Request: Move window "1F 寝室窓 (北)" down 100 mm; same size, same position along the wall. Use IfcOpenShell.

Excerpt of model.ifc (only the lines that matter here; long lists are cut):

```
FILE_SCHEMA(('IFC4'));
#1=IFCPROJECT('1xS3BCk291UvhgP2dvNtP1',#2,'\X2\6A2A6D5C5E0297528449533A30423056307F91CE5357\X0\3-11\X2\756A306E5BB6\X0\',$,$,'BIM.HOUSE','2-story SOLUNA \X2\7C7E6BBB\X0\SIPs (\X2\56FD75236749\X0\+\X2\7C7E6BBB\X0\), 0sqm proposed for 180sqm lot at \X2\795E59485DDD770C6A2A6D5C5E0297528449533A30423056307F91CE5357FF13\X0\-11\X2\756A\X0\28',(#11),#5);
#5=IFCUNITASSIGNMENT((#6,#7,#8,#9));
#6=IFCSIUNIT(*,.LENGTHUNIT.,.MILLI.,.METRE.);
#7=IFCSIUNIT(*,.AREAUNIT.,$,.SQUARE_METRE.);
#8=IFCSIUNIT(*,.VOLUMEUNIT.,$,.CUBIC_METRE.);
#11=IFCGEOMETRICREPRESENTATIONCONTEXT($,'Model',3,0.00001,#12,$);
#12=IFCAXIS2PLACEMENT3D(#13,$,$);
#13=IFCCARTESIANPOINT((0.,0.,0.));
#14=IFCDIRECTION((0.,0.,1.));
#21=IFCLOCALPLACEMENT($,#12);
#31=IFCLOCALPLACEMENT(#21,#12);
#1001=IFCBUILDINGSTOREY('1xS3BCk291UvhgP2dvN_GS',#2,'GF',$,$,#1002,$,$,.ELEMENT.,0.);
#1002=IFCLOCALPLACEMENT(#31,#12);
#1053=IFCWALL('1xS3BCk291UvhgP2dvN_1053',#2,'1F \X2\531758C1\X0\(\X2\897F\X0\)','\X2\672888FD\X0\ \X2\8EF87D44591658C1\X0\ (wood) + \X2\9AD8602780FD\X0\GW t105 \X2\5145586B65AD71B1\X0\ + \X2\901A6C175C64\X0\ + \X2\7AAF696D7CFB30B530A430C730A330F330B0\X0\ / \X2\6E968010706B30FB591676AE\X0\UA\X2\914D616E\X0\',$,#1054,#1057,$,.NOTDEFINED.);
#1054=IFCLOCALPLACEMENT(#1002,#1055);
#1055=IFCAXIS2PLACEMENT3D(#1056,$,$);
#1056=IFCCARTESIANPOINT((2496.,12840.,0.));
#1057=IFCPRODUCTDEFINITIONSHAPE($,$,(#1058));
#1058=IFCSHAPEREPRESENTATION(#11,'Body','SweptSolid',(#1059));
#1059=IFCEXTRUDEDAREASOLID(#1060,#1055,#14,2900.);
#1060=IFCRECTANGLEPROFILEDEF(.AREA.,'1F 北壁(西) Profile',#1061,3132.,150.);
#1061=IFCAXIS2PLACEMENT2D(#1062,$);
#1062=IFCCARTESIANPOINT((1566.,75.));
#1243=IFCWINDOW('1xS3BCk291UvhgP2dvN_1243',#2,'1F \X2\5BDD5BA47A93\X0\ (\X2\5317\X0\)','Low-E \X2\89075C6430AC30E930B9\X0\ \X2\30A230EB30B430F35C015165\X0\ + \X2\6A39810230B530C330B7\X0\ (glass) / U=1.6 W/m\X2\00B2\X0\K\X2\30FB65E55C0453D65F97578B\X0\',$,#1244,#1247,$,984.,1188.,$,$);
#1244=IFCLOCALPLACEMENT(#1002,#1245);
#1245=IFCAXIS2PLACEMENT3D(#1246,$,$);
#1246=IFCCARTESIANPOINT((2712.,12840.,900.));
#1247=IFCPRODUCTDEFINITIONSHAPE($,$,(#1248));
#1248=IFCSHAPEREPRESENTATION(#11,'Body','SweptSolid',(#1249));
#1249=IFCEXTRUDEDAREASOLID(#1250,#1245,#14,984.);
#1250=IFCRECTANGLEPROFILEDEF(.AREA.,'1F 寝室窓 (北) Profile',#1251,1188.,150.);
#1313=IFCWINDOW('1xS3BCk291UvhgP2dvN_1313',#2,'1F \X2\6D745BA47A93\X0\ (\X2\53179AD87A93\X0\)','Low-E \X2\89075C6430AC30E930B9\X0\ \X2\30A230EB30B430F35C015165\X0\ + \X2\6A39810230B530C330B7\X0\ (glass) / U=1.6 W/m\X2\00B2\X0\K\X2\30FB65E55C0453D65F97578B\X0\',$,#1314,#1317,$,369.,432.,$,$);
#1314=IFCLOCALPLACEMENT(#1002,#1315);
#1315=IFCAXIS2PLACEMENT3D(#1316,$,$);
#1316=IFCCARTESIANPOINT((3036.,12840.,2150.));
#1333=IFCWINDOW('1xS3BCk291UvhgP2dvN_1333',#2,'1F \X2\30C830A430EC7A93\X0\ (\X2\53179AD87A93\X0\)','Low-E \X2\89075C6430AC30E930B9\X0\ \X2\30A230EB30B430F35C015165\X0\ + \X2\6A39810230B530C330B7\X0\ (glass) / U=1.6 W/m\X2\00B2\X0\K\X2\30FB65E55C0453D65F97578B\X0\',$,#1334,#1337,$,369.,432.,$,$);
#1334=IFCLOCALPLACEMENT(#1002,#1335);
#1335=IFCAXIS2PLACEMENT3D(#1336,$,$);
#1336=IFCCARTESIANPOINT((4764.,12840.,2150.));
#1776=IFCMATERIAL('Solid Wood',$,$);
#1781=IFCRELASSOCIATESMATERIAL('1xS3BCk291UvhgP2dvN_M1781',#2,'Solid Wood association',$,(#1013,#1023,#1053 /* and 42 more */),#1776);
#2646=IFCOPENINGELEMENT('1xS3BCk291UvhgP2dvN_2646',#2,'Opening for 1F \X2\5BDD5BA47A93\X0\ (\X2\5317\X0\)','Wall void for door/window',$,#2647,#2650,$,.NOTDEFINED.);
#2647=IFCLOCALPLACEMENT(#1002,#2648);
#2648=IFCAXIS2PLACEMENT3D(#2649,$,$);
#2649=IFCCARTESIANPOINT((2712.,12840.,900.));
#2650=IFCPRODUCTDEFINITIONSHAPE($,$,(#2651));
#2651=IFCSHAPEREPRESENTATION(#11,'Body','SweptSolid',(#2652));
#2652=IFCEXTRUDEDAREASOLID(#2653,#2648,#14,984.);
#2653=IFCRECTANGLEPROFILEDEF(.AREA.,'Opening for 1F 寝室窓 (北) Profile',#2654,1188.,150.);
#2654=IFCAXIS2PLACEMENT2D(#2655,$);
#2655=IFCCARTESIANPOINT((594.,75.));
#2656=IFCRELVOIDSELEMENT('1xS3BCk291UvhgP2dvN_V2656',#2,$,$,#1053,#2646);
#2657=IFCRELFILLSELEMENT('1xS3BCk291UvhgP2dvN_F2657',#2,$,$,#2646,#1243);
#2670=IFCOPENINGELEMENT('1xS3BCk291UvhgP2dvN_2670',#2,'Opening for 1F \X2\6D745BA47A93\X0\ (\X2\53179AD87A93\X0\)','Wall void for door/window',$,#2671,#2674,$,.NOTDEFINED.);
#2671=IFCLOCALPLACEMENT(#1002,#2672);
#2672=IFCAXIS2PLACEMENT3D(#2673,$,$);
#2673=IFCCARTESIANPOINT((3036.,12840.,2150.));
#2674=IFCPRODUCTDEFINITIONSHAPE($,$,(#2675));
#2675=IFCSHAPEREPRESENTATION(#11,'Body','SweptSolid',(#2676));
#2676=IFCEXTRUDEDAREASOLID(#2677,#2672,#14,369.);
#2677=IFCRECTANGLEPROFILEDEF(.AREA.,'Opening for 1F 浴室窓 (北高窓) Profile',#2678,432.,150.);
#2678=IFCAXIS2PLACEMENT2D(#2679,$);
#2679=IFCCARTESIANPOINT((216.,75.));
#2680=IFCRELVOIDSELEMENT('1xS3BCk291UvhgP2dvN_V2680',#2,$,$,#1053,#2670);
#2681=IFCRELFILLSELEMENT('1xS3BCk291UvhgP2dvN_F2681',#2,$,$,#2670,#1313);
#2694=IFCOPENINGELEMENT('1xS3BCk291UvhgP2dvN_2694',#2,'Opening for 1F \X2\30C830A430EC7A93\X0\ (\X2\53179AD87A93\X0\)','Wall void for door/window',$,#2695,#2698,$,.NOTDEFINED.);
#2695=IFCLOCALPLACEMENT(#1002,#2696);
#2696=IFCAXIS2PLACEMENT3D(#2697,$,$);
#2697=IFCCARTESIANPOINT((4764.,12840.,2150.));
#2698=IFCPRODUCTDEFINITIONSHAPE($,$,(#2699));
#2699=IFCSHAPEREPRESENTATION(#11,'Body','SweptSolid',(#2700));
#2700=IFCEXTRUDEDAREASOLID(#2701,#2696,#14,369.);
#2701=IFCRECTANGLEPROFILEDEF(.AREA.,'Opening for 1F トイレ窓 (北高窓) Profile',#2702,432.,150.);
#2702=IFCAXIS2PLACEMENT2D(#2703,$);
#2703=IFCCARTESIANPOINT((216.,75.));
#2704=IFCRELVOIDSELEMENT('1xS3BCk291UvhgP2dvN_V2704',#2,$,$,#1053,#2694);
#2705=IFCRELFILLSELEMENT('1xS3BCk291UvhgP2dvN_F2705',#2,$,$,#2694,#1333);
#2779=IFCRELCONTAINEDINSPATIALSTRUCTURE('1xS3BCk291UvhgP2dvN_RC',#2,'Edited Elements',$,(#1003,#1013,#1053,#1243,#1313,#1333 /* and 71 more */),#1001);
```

```python
import numpy as np
import ifcopenshell
import ifcopenshell.api.geometry
import ifcopenshell.util.placement
import ifcopenshell.util.unit

model = ifcopenshell.open("model.ifc")
unit_scale = ifcopenshell.util.unit.calculate_unit_scale(model)

window = model.by_guid("1xS3BCk291UvhgP2dvN_1243")
opening = window.FillsVoids[0].RelatingOpeningElement
dz = -100.0

shift = np.array([0.0, 0.0, dz])
# The window is not placed relative to its opening, so move both.
for product in (opening, window):
    matrix = ifcopenshell.util.placement.get_local_placement(product.ObjectPlacement)
    matrix[:3, 3] += shift
    ifcopenshell.api.geometry.edit_object_placement(model, product=product, matrix=matrix, is_si=False)

print(f"moved by {dz * unit_scale:+.3f} m")

model.write("model_edited.ifc")
```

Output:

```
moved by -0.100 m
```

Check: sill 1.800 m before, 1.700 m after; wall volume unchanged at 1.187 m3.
